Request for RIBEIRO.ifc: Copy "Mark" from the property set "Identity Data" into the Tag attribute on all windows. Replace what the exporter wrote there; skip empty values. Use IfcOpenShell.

First a look at what the model holds.

```python
import ifcopenshell
import ifcopenshell.util.element

model = ifcopenshell.open("RIBEIRO.ifc")
print(model.schema)
windows = model.by_type("IfcWindow")
print(len(windows), "windows")
for e in windows[:8]:
    source = ifcopenshell.util.element.get_pset(e, "Identity Data", "Mark")
    target = e.Tag
    print(e.id(), repr(source), repr(target), sep=" | ")
```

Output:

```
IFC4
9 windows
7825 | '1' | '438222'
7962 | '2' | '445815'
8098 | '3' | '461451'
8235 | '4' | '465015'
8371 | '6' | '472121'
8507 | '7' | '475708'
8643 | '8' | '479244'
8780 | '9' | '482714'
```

```python
import ifcopenshell
import ifcopenshell.util.element

model = ifcopenshell.open("RIBEIRO.ifc")

count = 0
for e in model.by_type("IfcWindow"):
    value = ifcopenshell.util.element.get_pset(e, "Identity Data", "Mark")
    current = e.Tag
    if not value or not value.strip() or current == value:
        continue
    e.Tag = value
    count += 1

print(count, "windows updated")

model.write("RIBEIRO_updated.ifc")
```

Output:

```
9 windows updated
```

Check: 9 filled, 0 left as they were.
